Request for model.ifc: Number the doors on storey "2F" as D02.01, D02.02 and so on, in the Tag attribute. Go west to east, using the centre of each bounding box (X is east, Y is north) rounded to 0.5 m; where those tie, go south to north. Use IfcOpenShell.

First a look at what the model holds.

```python
import ifcopenshell
import ifcopenshell.util.element
import ifcopenshell.util.placement

model = ifcopenshell.open("model.ifc")
print(model.schema)
storey = next(s for s in model.by_type("IfcBuildingStorey") if s.Name == "2F")
doors = [e for e in ifcopenshell.util.element.get_decomposition(storey) if e.is_a("IfcDoor")]
for e in sorted(doors, key=lambda e: e.id()):
    origin = ifcopenshell.util.placement.get_local_placement(e.ObjectPlacement)[:3, 3]
    print(e.id(), e.Tag, e.Name, origin.round(2) + 0.0, sep=" | ")
```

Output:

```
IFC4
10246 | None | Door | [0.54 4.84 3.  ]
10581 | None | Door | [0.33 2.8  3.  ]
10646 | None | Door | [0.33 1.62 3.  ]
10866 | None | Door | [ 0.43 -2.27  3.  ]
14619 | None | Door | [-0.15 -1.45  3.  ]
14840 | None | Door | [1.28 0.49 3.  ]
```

```python
import ifcopenshell
import ifcopenshell.geom
import ifcopenshell.util.element
import ifcopenshell.util.shape

model = ifcopenshell.open("model.ifc")
settings = ifcopenshell.geom.settings()
settings.set("use-world-coords", True)


def centre(element):
    shape = ifcopenshell.geom.create_shape(settings, element)
    return ifcopenshell.util.shape.get_bbox_centroid(shape.geometry)


storey = next(s for s in model.by_type("IfcBuildingStorey") if s.Name == "2F")
doors = [e for e in ifcopenshell.util.element.get_decomposition(storey) if e.is_a("IfcDoor")]

# Insertion points can sit at a corner or the storey origin, so sort by the geometry (in metres).
centres = {e: centre(e) for e in doors}
doors.sort(key=lambda e: (round(centres[e][0] / 0.5), centres[e][1]))

for i, e in enumerate(doors, start=1):
    number = f"D02.{i:02d}"
    e.Tag = number
    print(e.id(), number)

model.write("model_v2.ifc")
```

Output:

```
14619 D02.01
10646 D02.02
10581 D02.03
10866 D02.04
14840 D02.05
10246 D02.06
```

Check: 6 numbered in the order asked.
